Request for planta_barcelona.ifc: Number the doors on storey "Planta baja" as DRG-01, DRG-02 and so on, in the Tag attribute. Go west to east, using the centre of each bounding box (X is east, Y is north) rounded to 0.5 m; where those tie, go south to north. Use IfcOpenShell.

First a look at what the model holds.

```python
import ifcopenshell
import ifcopenshell.util.element
import ifcopenshell.util.placement

model = ifcopenshell.open("planta_barcelona.ifc")
print(model.schema)
storey = next(s for s in model.by_type("IfcBuildingStorey") if s.Name == "Planta baja")
doors = [e for e in ifcopenshell.util.element.get_decomposition(storey) if e.is_a("IfcDoor")]
for e in sorted(doors, key=lambda e: e.id()):
    origin = ifcopenshell.util.placement.get_local_placement(e.ObjectPlacement)[:3, 3]
    print(e.id(), e.Tag, e.Name, origin.round(2) + 0.0, sep=" | ")
```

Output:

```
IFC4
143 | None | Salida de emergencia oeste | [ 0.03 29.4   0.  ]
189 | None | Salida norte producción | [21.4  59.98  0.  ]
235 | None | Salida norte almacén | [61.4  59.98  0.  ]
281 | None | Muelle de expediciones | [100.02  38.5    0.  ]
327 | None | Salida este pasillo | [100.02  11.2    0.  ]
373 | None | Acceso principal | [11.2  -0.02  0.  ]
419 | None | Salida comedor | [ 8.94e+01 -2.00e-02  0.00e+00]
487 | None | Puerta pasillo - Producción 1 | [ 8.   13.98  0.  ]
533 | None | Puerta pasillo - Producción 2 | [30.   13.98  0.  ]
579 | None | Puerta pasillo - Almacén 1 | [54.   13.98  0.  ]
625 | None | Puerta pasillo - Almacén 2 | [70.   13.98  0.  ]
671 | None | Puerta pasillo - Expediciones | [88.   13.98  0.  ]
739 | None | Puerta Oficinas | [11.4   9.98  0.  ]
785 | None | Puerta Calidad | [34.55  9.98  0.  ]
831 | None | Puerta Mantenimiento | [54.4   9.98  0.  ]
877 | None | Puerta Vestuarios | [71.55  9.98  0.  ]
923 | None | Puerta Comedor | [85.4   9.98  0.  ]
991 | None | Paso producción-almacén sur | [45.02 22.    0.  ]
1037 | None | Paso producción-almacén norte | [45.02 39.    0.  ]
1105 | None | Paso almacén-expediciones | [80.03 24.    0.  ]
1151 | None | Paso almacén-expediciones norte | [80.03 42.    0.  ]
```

```python
import ifcopenshell
import ifcopenshell.geom
import ifcopenshell.util.element
import ifcopenshell.util.shape

model = ifcopenshell.open("planta_barcelona.ifc")
settings = ifcopenshell.geom.settings()
settings.set("use-world-coords", True)


def centre(element):
    shape = ifcopenshell.geom.create_shape(settings, element)
    return ifcopenshell.util.shape.get_bbox_centroid(shape.geometry)


storey = next(s for s in model.by_type("IfcBuildingStorey") if s.Name == "Planta baja")
doors = [e for e in ifcopenshell.util.element.get_decomposition(storey) if e.is_a("IfcDoor")]

# Insertion points can sit at a corner or the storey origin, so sort by the geometry (in metres).
centres = {e: centre(e) for e in doors}
doors.sort(key=lambda e: (round(centres[e][0] / 0.5), centres[e][1]))

for i, e in enumerate(doors, start=1):
    number = f"DRG-{i:02d}"
    e.Tag = number
    print(e.id(), number)

model.write("planta_barcelona_rev.ifc")
```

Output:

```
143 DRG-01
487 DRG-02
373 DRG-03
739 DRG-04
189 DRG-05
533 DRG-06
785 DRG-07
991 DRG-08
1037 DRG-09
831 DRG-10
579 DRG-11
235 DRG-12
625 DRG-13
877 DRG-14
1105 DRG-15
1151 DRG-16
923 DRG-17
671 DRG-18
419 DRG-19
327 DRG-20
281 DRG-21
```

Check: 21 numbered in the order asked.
